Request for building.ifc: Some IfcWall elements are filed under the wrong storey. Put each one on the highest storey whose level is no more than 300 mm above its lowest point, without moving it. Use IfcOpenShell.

First a look at what the model holds.

```python
import ifcopenshell
import ifcopenshell.util.element
import ifcopenshell.util.placement

model = ifcopenshell.open("building.ifc")
print(model.schema)
for storey in model.by_type("IfcBuildingStorey"):
    level = ifcopenshell.util.placement.get_storey_elevation(storey)
    count = sum(e.is_a("IfcWall") for e in ifcopenshell.util.element.get_contained(storey))
    print(storey.id(), storey.Name, round(level, 3), count, sep=" | ")
```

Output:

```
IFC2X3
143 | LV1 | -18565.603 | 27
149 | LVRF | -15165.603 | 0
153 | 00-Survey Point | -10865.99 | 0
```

```python
import ifcopenshell
import ifcopenshell.api.spatial
import ifcopenshell.geom
import ifcopenshell.util.element
import ifcopenshell.util.placement
import ifcopenshell.util.shape
import ifcopenshell.util.unit

model = ifcopenshell.open("building.ifc")
unit_scale = ifcopenshell.util.unit.calculate_unit_scale(model)
settings = ifcopenshell.geom.settings()

levels = sorted(
    ((ifcopenshell.util.placement.get_storey_elevation(s) * unit_scale, s) for s in model.by_type("IfcBuildingStorey")),
    key=lambda pair: pair[0],
)

for e in model.by_type("IfcWall"):
    current = e.ContainedInStructure[0].RelatingStructure if e.ContainedInStructure else None
    if current is None or not current.is_a("IfcBuildingStorey"):
        continue
    shape = ifcopenshell.geom.create_shape(settings, e)
    bottom = ifcopenshell.util.shape.get_shape_bottom_elevation(shape, shape.geometry)
    below = [s for level, s in levels if level <= bottom + 0.3]
    storey = below[-1] if below else levels[0][1]
    if storey != current:
        # assign_container keeps the world position.
        ifcopenshell.api.spatial.assign_container(model, products=[e], relating_structure=storey)
        print(e.id(), current.Name, "->", storey.Name)

model.write("building_updated.ifc")
```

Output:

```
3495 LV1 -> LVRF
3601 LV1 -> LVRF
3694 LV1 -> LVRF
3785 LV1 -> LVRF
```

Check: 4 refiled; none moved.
